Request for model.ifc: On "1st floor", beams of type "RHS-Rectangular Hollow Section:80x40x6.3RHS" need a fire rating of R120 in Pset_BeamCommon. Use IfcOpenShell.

First a look at what the model holds.

```python
import ifcopenshell
import ifcopenshell.util.element

model = ifcopenshell.open("model.ifc")
print(model.schema)
storey = next(s for s in model.by_type("IfcBuildingStorey") if s.Name == "1st floor")
beams = [e for e in ifcopenshell.util.element.get_decomposition(storey) if e.is_a("IfcBeam")]
seen = {}
for e in beams:
    element_type = ifcopenshell.util.element.get_type(e)
    key = (element_type.Name if element_type != e and element_type else None, ifcopenshell.util.element.get_pset(e, "Pset_BeamCommon", "FireRating"))
    seen[key] = seen.get(key, 0) + 1
for (name, value), count in sorted(seen.items(), key=str):
    print(count, "x", name, "|", value)
```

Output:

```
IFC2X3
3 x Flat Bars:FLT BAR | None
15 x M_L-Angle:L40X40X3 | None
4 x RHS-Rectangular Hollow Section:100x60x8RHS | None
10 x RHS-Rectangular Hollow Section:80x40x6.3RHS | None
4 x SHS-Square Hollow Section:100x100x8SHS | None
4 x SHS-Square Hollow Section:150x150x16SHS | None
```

```python
import ifcopenshell
import ifcopenshell.api.pset
import ifcopenshell.util.element

model = ifcopenshell.open("model.ifc")

storey = next(s for s in model.by_type("IfcBuildingStorey") if s.Name == "1st floor")
beams = [e for e in ifcopenshell.util.element.get_decomposition(storey) if e.is_a("IfcBeam")]

count = 0
for e in beams:
    element_type = ifcopenshell.util.element.get_type(e)
    if element_type in (None, e) or element_type.Name != "RHS-Rectangular Hollow Section:80x40x6.3RHS":
        continue
    # add_pset returns the element's existing set when there is one.
    pset = ifcopenshell.api.pset.add_pset(model, product=e, name="Pset_BeamCommon")
    ifcopenshell.api.pset.edit_pset(model, pset=pset, properties={"FireRating": "R120"})
    count += 1

print(count, "beams updated")

model.write("model_edited.ifc")
```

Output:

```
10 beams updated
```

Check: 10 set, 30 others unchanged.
